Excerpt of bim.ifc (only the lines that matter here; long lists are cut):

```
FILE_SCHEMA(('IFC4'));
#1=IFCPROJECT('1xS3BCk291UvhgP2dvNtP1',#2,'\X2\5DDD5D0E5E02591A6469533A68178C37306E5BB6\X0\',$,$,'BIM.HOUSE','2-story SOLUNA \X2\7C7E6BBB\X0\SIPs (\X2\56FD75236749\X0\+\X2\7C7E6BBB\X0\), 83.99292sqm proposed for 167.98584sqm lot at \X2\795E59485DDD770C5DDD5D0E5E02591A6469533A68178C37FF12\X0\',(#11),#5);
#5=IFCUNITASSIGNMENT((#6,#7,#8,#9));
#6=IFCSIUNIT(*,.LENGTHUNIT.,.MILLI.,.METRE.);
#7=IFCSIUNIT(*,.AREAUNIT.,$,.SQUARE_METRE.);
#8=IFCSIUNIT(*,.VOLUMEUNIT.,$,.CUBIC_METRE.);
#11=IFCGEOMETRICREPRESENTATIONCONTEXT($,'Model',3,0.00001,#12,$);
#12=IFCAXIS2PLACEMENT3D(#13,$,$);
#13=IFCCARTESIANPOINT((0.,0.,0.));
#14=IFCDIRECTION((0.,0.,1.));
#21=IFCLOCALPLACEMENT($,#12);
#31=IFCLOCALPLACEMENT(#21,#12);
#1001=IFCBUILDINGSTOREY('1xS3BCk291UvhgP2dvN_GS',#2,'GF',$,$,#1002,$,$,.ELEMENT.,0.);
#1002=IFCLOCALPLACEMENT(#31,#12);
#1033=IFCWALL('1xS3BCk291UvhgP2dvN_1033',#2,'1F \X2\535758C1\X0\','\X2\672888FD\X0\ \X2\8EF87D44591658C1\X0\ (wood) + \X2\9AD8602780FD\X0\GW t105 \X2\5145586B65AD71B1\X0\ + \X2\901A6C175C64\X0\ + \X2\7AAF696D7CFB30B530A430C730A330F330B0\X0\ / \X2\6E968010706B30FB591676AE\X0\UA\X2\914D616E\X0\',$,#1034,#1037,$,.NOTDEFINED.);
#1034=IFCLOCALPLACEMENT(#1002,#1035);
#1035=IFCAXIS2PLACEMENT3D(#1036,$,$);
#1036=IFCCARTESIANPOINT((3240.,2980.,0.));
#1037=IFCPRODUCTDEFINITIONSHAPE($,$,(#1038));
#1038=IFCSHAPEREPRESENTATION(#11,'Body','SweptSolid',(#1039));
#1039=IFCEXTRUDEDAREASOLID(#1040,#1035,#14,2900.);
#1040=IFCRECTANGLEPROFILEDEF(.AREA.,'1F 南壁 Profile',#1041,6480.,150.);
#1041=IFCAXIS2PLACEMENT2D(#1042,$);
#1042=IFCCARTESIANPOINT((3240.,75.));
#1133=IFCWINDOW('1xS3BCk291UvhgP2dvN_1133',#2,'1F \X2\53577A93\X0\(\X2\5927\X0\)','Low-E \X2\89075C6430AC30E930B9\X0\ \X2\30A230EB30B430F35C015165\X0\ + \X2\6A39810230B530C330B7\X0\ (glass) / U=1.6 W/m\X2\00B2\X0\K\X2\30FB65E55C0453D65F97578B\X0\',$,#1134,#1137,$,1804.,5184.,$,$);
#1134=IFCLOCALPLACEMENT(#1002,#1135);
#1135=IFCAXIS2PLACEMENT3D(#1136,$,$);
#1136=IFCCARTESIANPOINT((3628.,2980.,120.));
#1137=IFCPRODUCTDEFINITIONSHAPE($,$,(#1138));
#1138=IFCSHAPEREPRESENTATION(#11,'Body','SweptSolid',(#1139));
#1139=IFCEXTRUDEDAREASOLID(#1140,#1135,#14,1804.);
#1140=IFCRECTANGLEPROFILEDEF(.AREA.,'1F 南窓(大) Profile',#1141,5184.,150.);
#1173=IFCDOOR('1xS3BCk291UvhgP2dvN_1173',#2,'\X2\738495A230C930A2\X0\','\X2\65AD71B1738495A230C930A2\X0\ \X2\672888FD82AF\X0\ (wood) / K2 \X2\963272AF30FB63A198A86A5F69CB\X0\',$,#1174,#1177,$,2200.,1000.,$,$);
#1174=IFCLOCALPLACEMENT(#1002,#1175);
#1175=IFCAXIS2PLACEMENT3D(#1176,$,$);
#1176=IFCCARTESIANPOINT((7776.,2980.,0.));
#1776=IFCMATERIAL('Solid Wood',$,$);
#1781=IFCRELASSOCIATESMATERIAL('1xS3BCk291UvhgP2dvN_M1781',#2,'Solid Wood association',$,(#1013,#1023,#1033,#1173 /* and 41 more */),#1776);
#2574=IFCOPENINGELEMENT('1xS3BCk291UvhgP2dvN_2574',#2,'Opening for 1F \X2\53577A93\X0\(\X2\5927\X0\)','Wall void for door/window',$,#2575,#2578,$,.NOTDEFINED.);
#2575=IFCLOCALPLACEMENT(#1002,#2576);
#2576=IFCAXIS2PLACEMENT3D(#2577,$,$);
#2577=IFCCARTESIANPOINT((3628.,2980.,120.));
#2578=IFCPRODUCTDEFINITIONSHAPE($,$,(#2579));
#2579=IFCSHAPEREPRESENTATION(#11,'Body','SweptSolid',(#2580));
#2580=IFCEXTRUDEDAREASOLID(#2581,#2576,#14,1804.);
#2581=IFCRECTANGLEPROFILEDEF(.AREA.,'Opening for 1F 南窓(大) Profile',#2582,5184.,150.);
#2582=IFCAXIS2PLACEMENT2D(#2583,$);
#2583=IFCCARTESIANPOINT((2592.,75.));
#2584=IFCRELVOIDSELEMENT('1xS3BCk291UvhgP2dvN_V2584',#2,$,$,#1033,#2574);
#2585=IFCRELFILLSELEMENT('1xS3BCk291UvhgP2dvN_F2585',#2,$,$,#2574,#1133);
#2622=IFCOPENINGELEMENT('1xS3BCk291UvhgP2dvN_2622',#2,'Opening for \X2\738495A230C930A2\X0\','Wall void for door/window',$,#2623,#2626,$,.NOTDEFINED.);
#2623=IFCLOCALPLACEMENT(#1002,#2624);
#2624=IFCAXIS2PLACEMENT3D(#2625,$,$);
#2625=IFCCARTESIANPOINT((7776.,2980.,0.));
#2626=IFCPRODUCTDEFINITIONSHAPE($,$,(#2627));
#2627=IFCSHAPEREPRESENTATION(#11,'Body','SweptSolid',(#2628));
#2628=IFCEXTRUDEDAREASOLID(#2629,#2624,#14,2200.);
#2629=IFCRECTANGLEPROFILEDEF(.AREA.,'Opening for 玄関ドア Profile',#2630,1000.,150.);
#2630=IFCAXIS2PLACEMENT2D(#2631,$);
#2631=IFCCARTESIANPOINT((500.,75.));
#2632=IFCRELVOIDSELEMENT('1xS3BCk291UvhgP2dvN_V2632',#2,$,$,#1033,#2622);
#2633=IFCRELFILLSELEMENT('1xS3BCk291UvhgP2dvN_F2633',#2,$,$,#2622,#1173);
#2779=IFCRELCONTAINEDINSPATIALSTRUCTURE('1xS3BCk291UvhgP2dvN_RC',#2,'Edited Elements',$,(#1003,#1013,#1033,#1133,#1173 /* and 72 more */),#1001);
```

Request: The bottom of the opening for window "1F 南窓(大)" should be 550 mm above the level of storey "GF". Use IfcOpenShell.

```python
import numpy as np
import ifcopenshell
import ifcopenshell.api.geometry
import ifcopenshell.geom
import ifcopenshell.util.element
import ifcopenshell.util.placement
import ifcopenshell.util.shape
import ifcopenshell.util.unit

model = ifcopenshell.open("bim.ifc")
unit_scale = ifcopenshell.util.unit.calculate_unit_scale(model)

window = model.by_guid("1xS3BCk291UvhgP2dvN_1133")
opening = window.FillsVoids[0].RelatingOpeningElement
storey = ifcopenshell.util.element.get_container(window, ifc_class="IfcBuildingStorey")
level = ifcopenshell.util.placement.get_local_placement(storey.ObjectPlacement)[2, 3]

# The opening's origin need not be at the sill, so measure its lowest point.
shape = ifcopenshell.geom.create_shape(ifcopenshell.geom.settings(), opening)
bottom = ifcopenshell.util.shape.get_shape_bottom_elevation(shape, shape.geometry) / unit_scale
dz = level + 0.55 / unit_scale - bottom

shift = np.array([0.0, 0.0, dz])
# The window is not placed relative to its opening, so move both.
for product in (opening, window):
    matrix = ifcopenshell.util.placement.get_local_placement(product.ObjectPlacement)
    matrix[:3, 3] += shift
    ifcopenshell.api.geometry.edit_object_placement(model, product=product, matrix=matrix, is_si=False)

print(f"moved by {dz * unit_scale:+.3f} m")

model.write("bim_edited.ifc")
```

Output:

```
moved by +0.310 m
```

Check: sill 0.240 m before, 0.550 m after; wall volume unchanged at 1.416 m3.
